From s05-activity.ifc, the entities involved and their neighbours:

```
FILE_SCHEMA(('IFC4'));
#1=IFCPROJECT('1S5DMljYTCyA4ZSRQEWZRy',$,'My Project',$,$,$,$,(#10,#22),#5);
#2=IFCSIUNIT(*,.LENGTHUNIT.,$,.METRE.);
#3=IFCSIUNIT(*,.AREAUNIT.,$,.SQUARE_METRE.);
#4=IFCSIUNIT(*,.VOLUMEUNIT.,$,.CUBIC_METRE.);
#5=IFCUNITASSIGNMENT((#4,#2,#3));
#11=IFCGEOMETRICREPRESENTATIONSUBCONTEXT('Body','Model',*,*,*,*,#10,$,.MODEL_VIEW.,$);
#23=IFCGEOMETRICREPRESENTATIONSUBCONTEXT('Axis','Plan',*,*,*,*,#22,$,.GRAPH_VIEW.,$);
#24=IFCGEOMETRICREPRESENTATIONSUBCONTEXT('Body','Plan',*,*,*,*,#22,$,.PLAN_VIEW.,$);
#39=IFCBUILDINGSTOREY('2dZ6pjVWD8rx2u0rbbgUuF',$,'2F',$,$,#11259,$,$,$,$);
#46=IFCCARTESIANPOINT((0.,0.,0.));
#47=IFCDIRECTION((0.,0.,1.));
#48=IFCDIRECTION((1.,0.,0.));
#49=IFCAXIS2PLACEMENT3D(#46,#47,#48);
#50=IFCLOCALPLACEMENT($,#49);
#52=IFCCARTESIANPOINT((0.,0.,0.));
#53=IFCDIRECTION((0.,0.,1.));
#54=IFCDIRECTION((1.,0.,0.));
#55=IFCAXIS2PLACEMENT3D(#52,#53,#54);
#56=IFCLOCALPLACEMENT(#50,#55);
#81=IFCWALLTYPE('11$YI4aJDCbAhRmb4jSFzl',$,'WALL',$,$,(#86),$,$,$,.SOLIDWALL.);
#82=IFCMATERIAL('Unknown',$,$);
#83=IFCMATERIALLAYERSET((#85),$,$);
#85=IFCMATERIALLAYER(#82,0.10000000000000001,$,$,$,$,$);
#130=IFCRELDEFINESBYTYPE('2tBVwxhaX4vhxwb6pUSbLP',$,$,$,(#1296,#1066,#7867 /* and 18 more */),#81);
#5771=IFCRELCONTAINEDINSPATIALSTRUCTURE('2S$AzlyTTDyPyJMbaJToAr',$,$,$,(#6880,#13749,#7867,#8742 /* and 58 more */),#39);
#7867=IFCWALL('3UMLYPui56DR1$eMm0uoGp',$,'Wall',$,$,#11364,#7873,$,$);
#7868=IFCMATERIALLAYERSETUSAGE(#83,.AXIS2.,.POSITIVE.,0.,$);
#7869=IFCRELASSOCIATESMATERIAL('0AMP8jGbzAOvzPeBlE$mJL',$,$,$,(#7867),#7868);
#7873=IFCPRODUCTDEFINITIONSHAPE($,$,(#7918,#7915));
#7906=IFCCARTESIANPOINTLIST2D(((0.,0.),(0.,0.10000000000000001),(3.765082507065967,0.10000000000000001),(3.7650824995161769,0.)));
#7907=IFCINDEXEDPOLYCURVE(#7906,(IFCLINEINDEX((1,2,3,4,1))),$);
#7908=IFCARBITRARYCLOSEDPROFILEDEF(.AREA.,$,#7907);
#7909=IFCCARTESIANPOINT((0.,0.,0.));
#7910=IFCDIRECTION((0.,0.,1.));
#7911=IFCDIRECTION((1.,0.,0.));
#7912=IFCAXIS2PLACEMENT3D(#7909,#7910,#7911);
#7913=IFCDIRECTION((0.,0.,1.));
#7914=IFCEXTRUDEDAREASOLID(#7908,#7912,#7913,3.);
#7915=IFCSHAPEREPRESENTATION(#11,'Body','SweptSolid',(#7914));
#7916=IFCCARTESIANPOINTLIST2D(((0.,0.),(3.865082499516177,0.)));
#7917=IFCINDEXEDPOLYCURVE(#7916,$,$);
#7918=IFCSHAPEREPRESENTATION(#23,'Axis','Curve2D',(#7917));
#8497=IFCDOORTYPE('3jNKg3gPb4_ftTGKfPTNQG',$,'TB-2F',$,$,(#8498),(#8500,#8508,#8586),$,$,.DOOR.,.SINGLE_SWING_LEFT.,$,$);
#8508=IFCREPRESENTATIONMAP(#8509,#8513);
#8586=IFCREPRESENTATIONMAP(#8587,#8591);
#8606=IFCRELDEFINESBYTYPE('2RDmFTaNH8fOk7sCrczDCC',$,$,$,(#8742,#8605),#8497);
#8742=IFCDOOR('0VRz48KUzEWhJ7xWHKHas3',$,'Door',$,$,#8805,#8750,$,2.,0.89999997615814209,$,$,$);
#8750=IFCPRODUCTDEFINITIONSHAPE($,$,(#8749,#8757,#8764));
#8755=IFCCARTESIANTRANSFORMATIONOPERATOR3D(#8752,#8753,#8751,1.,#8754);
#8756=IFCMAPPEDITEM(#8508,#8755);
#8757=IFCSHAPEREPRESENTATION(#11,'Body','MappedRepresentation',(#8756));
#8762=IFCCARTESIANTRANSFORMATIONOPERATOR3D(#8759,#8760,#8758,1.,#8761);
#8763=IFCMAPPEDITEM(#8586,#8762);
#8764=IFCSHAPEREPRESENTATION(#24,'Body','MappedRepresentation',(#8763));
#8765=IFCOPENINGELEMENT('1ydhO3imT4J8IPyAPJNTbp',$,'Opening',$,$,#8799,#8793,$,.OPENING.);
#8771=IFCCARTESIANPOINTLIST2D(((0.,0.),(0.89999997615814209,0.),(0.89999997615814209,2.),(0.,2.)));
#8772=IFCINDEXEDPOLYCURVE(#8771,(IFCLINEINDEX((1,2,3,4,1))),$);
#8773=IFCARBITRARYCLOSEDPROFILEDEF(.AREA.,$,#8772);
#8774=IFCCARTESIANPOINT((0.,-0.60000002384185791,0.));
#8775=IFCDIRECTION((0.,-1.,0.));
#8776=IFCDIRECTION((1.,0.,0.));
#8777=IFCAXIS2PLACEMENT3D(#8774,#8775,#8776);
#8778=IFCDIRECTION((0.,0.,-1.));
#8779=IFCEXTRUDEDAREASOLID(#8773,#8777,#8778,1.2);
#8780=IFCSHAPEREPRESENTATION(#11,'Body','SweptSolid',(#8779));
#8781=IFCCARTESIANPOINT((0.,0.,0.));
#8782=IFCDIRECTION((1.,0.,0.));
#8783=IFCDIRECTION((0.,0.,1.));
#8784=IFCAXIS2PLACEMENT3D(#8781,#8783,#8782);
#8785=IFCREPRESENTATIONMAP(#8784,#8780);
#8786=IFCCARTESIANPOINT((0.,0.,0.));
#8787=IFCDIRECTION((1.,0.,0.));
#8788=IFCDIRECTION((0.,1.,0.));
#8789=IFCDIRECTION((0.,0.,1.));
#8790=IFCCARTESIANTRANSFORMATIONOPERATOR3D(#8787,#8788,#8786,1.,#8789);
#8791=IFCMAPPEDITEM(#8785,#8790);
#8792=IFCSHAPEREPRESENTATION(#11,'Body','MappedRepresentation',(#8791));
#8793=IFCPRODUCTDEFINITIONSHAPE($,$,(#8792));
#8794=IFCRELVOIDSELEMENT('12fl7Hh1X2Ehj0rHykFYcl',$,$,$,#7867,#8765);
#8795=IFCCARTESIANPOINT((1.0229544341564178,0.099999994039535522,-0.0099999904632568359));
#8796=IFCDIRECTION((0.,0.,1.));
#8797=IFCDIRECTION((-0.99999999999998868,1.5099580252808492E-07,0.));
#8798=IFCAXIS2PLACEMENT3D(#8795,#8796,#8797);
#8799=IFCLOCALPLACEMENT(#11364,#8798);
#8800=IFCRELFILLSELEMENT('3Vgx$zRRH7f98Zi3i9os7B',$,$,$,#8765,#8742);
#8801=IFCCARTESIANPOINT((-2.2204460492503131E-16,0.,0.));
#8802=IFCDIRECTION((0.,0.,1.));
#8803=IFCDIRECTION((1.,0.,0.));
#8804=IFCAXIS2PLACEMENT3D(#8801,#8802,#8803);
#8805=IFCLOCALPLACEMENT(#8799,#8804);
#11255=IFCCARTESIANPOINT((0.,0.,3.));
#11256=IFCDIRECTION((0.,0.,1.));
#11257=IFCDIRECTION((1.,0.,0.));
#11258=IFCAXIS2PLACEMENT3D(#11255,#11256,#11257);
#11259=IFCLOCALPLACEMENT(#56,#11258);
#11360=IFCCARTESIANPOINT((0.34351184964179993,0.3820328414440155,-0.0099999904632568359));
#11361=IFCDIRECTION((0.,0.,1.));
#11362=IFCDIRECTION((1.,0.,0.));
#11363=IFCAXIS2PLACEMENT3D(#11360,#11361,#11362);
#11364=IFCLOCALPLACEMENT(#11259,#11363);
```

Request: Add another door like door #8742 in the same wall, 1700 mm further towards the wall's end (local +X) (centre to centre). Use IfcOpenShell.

```python
import ifcopenshell
import ifcopenshell.api.feature
import ifcopenshell.api.geometry
import ifcopenshell.api.root
import ifcopenshell.geom
import ifcopenshell.util.element
import ifcopenshell.util.placement
import ifcopenshell.util.shape
import ifcopenshell.util.unit

model = ifcopenshell.open("s05-activity.ifc")
unit_scale = ifcopenshell.util.unit.calculate_unit_scale(model)
settings = ifcopenshell.geom.settings()


def volume(element):
    """Net volume in cubic metres, openings subtracted."""
    shape = ifcopenshell.geom.create_shape(settings, element)
    return ifcopenshell.util.shape.get_volume(shape.geometry)


door = model.by_id(8742)
opening = door.FillsVoids[0].RelatingOpeningElement
wall = opening.VoidsElements[0].RelatingBuildingElement
before = volume(wall)
shift = ifcopenshell.util.placement.get_local_placement(wall.ObjectPlacement)[:3, 0] * 1.7 / unit_scale

# copy_class copies the void relationship, type, container and properties, but no geometry.
new_opening = ifcopenshell.api.root.copy_class(model, product=opening)
new_opening.Representation = ifcopenshell.util.element.copy_deep(
    model, opening.Representation, exclude=["IfcGeometricRepresentationContext", "IfcRepresentationMap"]
)
new_door = ifcopenshell.api.root.copy_class(model, product=door)
new_door.Representation = ifcopenshell.util.element.copy_deep(
    model, door.Representation, exclude=["IfcGeometricRepresentationContext", "IfcRepresentationMap"]
)
ifcopenshell.api.feature.add_filling(model, opening=new_opening, element=new_door)

for old, new in ((opening, new_opening), (door, new_door)):
    matrix = ifcopenshell.util.placement.get_local_placement(old.ObjectPlacement)
    matrix[:3, 3] += shift
    ifcopenshell.api.geometry.edit_object_placement(model, product=new, matrix=matrix, is_si=False)

after = volume(wall)

print(f"wall volume {before:.3f} -> {after:.3f} m3")

model.write("s05-activity_updated.ifc")
```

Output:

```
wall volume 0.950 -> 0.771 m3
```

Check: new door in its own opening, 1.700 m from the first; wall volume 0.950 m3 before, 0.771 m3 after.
